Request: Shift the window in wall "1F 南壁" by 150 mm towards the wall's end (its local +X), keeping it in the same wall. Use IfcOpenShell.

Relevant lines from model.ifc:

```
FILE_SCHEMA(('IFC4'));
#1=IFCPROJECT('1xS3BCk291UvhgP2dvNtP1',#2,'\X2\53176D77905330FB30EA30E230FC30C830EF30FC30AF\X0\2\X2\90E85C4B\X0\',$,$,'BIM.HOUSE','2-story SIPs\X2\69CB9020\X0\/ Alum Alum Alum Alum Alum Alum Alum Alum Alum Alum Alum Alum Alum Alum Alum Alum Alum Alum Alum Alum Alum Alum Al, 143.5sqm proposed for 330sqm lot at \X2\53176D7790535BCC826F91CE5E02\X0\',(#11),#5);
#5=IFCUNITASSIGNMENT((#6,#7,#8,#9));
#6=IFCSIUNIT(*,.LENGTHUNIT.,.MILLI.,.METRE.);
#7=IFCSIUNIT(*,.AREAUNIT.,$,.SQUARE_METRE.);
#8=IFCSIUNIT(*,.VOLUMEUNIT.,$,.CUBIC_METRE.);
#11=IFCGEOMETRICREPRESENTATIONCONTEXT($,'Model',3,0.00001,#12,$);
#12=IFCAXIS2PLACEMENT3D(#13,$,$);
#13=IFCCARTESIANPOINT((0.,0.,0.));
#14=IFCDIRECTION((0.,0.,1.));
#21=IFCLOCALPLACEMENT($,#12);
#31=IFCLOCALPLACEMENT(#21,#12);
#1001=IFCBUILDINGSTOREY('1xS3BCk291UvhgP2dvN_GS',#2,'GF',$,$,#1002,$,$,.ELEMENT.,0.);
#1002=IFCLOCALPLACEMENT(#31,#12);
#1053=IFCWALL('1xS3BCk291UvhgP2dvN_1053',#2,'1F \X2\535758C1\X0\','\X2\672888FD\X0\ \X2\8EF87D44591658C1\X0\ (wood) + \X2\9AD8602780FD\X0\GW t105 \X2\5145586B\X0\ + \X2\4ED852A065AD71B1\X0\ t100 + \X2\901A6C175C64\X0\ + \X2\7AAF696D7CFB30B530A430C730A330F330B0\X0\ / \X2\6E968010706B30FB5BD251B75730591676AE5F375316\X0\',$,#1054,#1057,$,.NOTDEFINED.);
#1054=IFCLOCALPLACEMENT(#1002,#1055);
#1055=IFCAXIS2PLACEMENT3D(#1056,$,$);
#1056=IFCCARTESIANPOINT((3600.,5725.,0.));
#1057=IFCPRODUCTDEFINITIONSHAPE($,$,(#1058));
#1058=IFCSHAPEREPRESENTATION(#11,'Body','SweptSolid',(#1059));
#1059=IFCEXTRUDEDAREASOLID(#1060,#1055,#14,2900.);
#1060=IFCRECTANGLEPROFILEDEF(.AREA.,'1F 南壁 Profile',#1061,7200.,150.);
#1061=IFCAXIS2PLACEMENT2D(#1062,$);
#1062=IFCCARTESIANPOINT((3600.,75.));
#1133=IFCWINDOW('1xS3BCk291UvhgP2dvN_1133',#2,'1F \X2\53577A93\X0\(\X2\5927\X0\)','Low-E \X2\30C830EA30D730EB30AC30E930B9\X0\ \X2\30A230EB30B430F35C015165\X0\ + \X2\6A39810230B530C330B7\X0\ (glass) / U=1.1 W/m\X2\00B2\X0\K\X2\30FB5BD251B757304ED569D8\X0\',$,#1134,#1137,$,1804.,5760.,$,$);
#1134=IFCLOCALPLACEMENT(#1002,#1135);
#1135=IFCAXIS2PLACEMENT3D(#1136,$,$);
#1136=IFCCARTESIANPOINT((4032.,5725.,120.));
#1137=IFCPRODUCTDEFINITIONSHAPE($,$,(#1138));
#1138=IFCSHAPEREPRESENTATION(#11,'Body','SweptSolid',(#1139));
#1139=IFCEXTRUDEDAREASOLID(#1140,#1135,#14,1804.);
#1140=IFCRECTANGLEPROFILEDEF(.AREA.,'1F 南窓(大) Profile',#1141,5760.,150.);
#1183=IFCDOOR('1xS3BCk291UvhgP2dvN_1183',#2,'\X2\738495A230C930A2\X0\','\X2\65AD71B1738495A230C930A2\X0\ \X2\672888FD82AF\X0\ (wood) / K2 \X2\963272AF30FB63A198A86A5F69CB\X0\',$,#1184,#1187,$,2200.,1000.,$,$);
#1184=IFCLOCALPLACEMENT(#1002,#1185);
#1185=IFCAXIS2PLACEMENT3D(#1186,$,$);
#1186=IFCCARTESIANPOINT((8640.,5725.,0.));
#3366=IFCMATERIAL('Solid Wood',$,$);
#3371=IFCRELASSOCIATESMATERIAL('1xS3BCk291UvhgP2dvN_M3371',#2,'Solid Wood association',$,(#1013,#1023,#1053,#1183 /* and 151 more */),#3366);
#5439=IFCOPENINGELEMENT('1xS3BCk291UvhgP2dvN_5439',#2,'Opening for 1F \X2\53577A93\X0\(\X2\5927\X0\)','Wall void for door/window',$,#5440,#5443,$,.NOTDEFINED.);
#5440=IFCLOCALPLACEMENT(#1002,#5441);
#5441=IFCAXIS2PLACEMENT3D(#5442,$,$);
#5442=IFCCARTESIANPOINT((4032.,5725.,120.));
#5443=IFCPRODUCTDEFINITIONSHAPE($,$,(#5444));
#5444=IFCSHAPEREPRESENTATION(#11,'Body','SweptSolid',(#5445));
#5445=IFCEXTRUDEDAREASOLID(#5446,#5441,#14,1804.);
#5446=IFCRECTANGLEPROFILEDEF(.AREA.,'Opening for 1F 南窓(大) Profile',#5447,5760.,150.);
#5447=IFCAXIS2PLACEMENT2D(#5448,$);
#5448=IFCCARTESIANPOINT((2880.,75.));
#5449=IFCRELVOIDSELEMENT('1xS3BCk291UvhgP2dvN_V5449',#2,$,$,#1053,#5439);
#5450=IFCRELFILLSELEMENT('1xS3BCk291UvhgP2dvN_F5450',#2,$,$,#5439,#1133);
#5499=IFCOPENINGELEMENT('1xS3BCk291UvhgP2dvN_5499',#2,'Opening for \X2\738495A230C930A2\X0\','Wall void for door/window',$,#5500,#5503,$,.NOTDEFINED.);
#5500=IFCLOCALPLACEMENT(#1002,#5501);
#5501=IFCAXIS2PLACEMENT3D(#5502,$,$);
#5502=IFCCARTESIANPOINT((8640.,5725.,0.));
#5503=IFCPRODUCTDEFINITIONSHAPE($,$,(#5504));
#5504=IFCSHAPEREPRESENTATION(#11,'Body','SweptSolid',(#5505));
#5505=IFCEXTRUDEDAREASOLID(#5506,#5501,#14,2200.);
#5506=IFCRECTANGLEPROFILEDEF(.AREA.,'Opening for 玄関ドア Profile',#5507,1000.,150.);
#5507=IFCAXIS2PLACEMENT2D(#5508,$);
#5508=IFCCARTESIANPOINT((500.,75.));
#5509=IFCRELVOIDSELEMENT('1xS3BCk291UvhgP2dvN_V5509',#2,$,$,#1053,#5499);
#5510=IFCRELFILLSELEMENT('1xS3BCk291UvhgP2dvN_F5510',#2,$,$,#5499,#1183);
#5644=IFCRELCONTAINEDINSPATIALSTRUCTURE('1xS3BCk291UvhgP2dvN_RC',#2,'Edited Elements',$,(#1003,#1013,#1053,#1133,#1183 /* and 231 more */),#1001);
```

```python
import ifcopenshell
import ifcopenshell.api.geometry
import ifcopenshell.util.placement
import ifcopenshell.util.unit

model = ifcopenshell.open("model.ifc")
unit_scale = ifcopenshell.util.unit.calculate_unit_scale(model)

window = model.by_guid("1xS3BCk291UvhgP2dvN_1133")
opening = window.FillsVoids[0].RelatingOpeningElement
wall = opening.VoidsElements[0].RelatingBuildingElement

wall_matrix = ifcopenshell.util.placement.get_local_placement(wall.ObjectPlacement)
shift = wall_matrix[:3, 0] * 0.15 / unit_scale
before = ifcopenshell.util.placement.get_local_placement(window.ObjectPlacement)[:3, 3].copy()

# The window is not placed relative to its opening, so move both.
for product in (opening, window):
    matrix = ifcopenshell.util.placement.get_local_placement(product.ObjectPlacement)
    matrix[:3, 3] += shift
    ifcopenshell.api.geometry.edit_object_placement(model, product=product, matrix=matrix, is_si=False)

after = ifcopenshell.util.placement.get_local_placement(window.ObjectPlacement)[:3, 3]
print("window moved by", (after - before).round(3) + 0.0)

model.write("model_updated.ifc")
```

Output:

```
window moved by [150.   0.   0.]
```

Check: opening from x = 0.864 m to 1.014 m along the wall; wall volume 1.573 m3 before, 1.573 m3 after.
